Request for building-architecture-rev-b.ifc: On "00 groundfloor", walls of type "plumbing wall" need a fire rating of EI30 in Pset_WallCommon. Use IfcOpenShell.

First a look at what the model holds.

```python
import ifcopenshell
import ifcopenshell.util.element

model = ifcopenshell.open("building-architecture-rev-b.ifc")
print(model.schema)
storey = next(s for s in model.by_type("IfcBuildingStorey") if s.Name == "00 groundfloor")
walls = [e for e in ifcopenshell.util.element.get_decomposition(storey) if e.is_a("IfcWall")]
seen = {}
for e in walls:
    element_type = ifcopenshell.util.element.get_type(e)
    key = (element_type.Name if element_type != e and element_type else None, ifcopenshell.util.element.get_pset(e, "Pset_WallCommon", "FireRating"))
    seen[key] = seen.get(key, 0) + 1
for (name, value), count in sorted(seen.items(), key=str):
    print(count, "x", name, "|", value)
```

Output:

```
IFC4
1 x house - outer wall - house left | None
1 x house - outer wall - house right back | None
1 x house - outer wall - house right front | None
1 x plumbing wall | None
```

```python
import ifcopenshell
import ifcopenshell.api.pset
import ifcopenshell.util.element

model = ifcopenshell.open("building-architecture-rev-b.ifc")

storey = next(s for s in model.by_type("IfcBuildingStorey") if s.Name == "00 groundfloor")
walls = [e for e in ifcopenshell.util.element.get_decomposition(storey) if e.is_a("IfcWall")]

count = 0
for e in walls:
    element_type = ifcopenshell.util.element.get_type(e)
    if element_type in (None, e) or element_type.Name != "plumbing wall":
        continue
    # add_pset returns the element's existing set when there is one.
    pset = ifcopenshell.api.pset.add_pset(model, product=e, name="Pset_WallCommon")
    ifcopenshell.api.pset.edit_pset(model, pset=pset, properties={"FireRating": "EI30"})
    count += 1

print(count, "walls updated")

model.write("building-architecture-rev-b_updated.ifc")
```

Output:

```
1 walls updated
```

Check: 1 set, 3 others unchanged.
